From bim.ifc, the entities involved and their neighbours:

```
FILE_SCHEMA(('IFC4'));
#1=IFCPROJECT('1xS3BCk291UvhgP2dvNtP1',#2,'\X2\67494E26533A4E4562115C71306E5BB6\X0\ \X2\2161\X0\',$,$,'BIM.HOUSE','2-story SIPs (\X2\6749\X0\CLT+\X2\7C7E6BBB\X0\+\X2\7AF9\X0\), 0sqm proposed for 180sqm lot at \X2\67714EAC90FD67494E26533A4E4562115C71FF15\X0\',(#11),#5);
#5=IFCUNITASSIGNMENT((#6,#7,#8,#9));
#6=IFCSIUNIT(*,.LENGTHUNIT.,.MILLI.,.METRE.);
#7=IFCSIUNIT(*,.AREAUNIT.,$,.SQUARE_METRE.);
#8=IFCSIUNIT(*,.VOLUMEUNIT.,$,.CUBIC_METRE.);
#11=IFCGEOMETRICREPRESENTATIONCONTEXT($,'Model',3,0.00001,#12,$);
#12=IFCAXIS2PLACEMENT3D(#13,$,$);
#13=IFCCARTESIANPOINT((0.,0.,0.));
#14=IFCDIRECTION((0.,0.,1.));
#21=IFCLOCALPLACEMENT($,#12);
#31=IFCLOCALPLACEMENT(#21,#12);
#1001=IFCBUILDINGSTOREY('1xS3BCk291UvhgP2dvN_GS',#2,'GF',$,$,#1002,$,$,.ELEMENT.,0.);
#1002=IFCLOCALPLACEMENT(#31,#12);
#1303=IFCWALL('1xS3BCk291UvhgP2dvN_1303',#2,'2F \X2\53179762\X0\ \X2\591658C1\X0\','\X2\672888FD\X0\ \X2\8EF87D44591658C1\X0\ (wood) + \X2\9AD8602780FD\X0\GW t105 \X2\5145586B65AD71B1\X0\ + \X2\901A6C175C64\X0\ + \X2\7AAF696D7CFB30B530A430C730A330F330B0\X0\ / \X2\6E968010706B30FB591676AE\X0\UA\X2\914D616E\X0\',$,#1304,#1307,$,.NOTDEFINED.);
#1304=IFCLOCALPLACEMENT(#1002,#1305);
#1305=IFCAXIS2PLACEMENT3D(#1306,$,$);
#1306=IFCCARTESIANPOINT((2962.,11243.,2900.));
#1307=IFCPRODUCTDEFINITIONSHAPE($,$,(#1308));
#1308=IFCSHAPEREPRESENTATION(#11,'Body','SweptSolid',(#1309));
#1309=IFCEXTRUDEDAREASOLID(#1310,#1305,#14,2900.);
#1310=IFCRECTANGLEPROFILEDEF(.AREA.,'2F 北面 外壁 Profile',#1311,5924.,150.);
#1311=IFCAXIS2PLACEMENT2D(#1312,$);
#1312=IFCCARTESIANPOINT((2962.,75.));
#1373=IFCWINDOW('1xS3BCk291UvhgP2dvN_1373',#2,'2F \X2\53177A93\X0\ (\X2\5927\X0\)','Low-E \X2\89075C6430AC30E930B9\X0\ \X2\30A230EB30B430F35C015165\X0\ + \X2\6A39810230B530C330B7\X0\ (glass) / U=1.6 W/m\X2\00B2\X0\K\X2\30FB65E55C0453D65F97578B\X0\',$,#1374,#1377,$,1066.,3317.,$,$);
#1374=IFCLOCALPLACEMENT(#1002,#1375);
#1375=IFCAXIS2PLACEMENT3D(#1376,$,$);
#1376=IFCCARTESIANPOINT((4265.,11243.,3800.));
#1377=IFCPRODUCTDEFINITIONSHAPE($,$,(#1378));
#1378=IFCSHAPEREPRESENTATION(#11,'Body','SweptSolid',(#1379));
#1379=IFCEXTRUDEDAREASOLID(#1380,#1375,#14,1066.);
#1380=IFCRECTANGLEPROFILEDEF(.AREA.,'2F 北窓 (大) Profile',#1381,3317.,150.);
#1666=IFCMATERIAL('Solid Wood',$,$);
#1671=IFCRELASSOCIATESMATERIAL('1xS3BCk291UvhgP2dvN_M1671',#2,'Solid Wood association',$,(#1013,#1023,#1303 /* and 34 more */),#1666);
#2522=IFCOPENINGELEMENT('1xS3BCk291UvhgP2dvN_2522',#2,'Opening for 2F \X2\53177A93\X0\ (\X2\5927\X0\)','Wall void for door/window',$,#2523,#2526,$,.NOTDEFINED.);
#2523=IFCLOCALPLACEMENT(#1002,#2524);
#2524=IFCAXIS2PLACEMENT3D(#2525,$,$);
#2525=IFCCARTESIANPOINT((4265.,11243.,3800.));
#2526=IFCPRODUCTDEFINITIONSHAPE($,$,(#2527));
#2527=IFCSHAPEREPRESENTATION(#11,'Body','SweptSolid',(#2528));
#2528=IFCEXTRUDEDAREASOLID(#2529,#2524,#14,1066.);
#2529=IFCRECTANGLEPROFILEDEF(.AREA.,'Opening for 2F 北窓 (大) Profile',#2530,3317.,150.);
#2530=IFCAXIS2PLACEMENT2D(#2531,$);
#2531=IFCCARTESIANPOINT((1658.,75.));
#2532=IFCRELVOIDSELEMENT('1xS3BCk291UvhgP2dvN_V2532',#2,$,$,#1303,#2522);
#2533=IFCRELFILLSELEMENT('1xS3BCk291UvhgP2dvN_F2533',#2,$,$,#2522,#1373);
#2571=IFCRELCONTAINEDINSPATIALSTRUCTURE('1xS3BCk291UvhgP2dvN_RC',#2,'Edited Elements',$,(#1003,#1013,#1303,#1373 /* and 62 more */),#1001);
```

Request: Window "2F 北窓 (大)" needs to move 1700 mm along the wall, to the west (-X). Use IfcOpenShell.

```python
import ifcopenshell
import ifcopenshell.api.geometry
import ifcopenshell.util.placement

model = ifcopenshell.open("bim.ifc")

window = model.by_id(1373)
opening = window.FillsVoids[0].RelatingOpeningElement
wall = opening.VoidsElements[0].RelatingBuildingElement

wall_matrix = ifcopenshell.util.placement.get_local_placement(wall.ObjectPlacement)
shift = wall_matrix[:3, 0] * -1700.0
before = ifcopenshell.util.placement.get_local_placement(window.ObjectPlacement)[:3, 3].copy()

# The window is not placed relative to its opening, so move both.
for product in (opening, window):
    matrix = ifcopenshell.util.placement.get_local_placement(product.ObjectPlacement)
    matrix[:3, 3] += shift
    ifcopenshell.api.geometry.edit_object_placement(model, product=product, matrix=matrix, is_si=False)

after = ifcopenshell.util.placement.get_local_placement(window.ObjectPlacement)[:3, 3]
print("window moved by", (after - before).round(3) + 0.0)

model.write("bim_edited.ifc")
```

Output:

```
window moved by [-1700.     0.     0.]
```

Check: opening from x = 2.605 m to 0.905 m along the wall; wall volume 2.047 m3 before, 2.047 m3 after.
